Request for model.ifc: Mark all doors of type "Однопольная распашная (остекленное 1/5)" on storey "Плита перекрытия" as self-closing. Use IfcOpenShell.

First a look at what the model holds.

```python
import ifcopenshell
import ifcopenshell.util.element

model = ifcopenshell.open("model.ifc")
print(model.schema)
storey = next(s for s in model.by_type("IfcBuildingStorey") if s.Name == "Плита перекрытия")
doors = [e for e in ifcopenshell.util.element.get_decomposition(storey) if e.is_a("IfcDoor")]
seen = {}
for e in doors:
    element_type = ifcopenshell.util.element.get_type(e)
    key = (element_type.Name if element_type != e and element_type else None, ifcopenshell.util.element.get_pset(e, "Pset_DoorCommon", "SelfClosing"))
    seen[key] = seen.get(key, 0) + 1
for (name, value), count in sorted(seen.items(), key=str):
    print(count, "x", name, "|", value)
```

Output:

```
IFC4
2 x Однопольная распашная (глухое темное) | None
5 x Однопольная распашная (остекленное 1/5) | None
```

```python
import ifcopenshell
import ifcopenshell.api.pset
import ifcopenshell.util.element

model = ifcopenshell.open("model.ifc")

storey = next(s for s in model.by_type("IfcBuildingStorey") if s.Name == "Плита перекрытия")
doors = [e for e in ifcopenshell.util.element.get_decomposition(storey) if e.is_a("IfcDoor")]

count = 0
for e in doors:
    element_type = ifcopenshell.util.element.get_type(e)
    if element_type in (None, e) or element_type.Name != "Однопольная распашная (остекленное 1/5)":
        continue
    # add_pset returns the element's existing set when there is one.
    pset = ifcopenshell.api.pset.add_pset(model, product=e, name="Pset_DoorCommon")
    ifcopenshell.api.pset.edit_pset(model, pset=pset, properties={"SelfClosing": True})
    count += 1

print(count, "doors updated")

model.write("model_rev.ifc")
```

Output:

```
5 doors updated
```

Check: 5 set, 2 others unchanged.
